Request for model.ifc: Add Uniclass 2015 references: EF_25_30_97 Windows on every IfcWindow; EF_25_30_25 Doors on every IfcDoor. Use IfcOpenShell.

First a look at what the model holds.

```python
import ifcopenshell

model = ifcopenshell.open("model.ifc")
print(model.schema)
print("classifications:", [c.Name for c in model.by_type("IfcClassification")])
for ifc_class in ("IfcDoor", "IfcRoof", "IfcStair", "IfcWall", "IfcWindow"):
    print(ifc_class, len(model.by_type(ifc_class)))
```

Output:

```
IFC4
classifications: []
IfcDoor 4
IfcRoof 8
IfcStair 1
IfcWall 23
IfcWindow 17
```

```python
import ifcopenshell
import ifcopenshell.api.classification

model = ifcopenshell.open("model.ifc")

system = ifcopenshell.api.classification.add_classification(model, classification="Uniclass 2015")

codes = {
    "IfcWindow": ("EF_25_30_97", "Windows"),
    "IfcDoor": ("EF_25_30_25", "Doors"),
}
for ifc_class, (code, name) in codes.items():
    products = model.by_type(ifc_class)
    ifcopenshell.api.classification.add_reference(
        model, products=products, classification=system, identification=code, name=name
    )
    print(code, len(products))

model.write("model_v2.ifc")
```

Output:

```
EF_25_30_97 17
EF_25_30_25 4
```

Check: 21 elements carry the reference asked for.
